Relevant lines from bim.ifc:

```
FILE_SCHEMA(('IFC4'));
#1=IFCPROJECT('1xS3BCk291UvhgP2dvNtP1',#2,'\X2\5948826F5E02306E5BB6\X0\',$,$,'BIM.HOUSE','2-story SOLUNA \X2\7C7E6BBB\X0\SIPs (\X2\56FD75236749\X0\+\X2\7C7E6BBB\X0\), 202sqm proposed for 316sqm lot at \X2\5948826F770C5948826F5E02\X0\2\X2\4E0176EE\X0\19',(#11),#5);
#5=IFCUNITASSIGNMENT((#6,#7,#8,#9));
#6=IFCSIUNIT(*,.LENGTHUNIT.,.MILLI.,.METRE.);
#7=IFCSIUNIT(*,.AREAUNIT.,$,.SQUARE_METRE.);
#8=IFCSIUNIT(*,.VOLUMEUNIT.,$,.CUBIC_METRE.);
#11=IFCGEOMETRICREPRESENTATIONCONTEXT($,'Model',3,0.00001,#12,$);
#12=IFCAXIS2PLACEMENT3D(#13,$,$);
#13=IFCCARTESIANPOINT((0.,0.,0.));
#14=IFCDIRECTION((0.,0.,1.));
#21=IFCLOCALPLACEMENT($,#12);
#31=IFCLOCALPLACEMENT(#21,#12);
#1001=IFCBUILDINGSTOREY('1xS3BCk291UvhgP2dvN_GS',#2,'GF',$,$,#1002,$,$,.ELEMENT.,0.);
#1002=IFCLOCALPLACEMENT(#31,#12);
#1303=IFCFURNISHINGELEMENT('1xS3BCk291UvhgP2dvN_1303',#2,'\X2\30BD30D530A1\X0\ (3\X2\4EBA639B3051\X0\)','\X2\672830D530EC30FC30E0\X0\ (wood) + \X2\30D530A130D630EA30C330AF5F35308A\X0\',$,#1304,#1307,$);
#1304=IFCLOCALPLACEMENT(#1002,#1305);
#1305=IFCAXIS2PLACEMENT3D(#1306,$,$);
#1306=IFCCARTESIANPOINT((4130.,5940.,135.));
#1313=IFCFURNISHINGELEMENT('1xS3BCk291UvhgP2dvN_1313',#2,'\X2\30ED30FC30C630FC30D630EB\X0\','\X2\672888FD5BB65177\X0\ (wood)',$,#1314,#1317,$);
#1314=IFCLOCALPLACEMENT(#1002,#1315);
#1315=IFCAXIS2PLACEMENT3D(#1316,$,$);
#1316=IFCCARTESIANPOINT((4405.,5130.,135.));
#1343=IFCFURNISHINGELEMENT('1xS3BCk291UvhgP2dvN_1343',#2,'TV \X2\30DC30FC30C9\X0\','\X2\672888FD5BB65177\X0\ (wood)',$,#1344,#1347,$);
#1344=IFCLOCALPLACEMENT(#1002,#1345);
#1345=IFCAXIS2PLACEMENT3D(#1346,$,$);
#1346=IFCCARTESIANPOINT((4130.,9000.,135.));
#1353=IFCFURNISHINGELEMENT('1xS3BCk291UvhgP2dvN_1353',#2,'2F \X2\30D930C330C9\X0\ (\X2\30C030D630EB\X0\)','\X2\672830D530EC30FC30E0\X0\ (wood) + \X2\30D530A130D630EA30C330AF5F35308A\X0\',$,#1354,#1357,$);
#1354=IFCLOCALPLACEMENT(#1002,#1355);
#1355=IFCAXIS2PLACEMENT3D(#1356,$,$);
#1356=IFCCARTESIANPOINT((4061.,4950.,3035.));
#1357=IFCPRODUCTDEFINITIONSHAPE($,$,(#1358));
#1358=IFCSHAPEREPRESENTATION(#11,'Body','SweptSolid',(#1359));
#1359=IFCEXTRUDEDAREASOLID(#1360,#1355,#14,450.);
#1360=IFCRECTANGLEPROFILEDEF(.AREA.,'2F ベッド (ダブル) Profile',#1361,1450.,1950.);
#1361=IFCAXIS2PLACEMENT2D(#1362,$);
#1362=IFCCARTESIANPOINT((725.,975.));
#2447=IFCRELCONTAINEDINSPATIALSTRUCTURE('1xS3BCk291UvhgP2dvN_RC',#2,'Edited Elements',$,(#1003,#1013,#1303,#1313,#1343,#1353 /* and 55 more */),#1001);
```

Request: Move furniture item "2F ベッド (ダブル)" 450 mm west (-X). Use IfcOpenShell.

```python
import ifcopenshell
import ifcopenshell.api.geometry
import ifcopenshell.util.placement
import ifcopenshell.util.unit

model = ifcopenshell.open("bim.ifc")
unit_scale = ifcopenshell.util.unit.calculate_unit_scale(model)

item = model.by_id(1353)
matrix = ifcopenshell.util.placement.get_local_placement(item.ObjectPlacement)
matrix[0, 3] -= 0.45 / unit_scale
ifcopenshell.api.geometry.edit_object_placement(model, product=item, matrix=matrix, is_si=False)

print(ifcopenshell.util.placement.get_local_placement(item.ObjectPlacement).round(3) + 0.0)

model.write("bim_v2.ifc")
```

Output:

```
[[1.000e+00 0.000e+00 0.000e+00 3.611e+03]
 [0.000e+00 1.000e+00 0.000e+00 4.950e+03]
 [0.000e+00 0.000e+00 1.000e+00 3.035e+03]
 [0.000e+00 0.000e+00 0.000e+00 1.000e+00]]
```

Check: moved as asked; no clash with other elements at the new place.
